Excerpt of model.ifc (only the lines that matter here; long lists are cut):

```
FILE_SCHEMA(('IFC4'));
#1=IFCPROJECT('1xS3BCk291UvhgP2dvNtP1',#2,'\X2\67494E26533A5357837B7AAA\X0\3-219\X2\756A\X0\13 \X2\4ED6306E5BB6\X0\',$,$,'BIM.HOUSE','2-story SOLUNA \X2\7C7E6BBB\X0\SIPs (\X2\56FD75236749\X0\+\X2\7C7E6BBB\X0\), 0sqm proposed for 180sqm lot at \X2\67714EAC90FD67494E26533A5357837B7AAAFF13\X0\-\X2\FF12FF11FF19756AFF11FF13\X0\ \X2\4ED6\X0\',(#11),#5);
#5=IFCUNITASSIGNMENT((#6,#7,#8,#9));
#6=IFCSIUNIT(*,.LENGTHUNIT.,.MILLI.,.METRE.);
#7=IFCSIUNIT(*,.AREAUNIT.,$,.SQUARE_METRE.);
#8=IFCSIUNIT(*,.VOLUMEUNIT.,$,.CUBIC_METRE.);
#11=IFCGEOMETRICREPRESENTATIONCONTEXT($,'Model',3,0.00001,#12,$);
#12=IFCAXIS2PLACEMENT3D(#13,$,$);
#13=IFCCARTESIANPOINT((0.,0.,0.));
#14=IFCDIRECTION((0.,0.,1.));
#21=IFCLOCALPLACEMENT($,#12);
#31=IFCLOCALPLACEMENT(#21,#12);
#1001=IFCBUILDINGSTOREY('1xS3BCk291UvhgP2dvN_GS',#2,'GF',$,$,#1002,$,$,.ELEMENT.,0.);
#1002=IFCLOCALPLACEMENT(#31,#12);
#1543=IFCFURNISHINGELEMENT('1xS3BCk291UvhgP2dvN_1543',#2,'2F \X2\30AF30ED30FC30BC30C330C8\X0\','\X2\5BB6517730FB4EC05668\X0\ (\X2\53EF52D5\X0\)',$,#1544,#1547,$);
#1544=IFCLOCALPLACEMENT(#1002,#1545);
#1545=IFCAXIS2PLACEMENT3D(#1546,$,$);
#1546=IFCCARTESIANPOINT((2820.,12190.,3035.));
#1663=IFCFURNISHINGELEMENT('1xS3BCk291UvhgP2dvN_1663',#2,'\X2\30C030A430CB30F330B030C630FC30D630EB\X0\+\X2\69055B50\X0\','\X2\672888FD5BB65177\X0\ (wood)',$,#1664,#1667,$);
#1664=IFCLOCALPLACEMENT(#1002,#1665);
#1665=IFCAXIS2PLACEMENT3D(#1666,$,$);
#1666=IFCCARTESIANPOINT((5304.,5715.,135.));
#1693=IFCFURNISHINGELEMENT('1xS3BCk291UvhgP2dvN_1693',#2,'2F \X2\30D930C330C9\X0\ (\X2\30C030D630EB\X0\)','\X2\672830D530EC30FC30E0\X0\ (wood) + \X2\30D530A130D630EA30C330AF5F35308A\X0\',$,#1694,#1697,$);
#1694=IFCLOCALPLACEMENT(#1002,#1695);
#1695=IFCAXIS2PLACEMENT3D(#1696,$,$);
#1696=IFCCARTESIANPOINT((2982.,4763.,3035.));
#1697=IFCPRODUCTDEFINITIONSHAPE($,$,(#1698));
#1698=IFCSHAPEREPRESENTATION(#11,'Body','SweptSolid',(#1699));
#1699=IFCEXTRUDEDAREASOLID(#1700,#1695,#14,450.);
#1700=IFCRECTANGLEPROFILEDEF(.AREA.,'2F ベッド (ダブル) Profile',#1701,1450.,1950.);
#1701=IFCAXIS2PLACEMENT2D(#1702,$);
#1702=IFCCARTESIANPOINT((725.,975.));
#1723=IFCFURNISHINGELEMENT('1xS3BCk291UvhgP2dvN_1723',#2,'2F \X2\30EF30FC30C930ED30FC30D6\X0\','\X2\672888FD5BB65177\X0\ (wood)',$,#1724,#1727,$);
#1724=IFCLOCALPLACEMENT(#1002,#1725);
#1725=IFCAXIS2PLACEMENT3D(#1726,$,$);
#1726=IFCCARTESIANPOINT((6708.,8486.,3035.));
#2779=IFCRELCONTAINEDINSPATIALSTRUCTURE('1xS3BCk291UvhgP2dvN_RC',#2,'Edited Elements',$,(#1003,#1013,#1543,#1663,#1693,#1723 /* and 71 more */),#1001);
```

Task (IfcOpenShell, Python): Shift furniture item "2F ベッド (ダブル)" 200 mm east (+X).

```python
import ifcopenshell
import ifcopenshell.api.geometry
import ifcopenshell.util.placement
import ifcopenshell.util.unit

model = ifcopenshell.open("model.ifc")
unit_scale = ifcopenshell.util.unit.calculate_unit_scale(model)

item = model.by_id(1693)
matrix = ifcopenshell.util.placement.get_local_placement(item.ObjectPlacement)
matrix[0, 3] += 0.2 / unit_scale
ifcopenshell.api.geometry.edit_object_placement(model, product=item, matrix=matrix, is_si=False)

print(ifcopenshell.util.placement.get_local_placement(item.ObjectPlacement).round(3) + 0.0)

model.write("model_edited.ifc")
```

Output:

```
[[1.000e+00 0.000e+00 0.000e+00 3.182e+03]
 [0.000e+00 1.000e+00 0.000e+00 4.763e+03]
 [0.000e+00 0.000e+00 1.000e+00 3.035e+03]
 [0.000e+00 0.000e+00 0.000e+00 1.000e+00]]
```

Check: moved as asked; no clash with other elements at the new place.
